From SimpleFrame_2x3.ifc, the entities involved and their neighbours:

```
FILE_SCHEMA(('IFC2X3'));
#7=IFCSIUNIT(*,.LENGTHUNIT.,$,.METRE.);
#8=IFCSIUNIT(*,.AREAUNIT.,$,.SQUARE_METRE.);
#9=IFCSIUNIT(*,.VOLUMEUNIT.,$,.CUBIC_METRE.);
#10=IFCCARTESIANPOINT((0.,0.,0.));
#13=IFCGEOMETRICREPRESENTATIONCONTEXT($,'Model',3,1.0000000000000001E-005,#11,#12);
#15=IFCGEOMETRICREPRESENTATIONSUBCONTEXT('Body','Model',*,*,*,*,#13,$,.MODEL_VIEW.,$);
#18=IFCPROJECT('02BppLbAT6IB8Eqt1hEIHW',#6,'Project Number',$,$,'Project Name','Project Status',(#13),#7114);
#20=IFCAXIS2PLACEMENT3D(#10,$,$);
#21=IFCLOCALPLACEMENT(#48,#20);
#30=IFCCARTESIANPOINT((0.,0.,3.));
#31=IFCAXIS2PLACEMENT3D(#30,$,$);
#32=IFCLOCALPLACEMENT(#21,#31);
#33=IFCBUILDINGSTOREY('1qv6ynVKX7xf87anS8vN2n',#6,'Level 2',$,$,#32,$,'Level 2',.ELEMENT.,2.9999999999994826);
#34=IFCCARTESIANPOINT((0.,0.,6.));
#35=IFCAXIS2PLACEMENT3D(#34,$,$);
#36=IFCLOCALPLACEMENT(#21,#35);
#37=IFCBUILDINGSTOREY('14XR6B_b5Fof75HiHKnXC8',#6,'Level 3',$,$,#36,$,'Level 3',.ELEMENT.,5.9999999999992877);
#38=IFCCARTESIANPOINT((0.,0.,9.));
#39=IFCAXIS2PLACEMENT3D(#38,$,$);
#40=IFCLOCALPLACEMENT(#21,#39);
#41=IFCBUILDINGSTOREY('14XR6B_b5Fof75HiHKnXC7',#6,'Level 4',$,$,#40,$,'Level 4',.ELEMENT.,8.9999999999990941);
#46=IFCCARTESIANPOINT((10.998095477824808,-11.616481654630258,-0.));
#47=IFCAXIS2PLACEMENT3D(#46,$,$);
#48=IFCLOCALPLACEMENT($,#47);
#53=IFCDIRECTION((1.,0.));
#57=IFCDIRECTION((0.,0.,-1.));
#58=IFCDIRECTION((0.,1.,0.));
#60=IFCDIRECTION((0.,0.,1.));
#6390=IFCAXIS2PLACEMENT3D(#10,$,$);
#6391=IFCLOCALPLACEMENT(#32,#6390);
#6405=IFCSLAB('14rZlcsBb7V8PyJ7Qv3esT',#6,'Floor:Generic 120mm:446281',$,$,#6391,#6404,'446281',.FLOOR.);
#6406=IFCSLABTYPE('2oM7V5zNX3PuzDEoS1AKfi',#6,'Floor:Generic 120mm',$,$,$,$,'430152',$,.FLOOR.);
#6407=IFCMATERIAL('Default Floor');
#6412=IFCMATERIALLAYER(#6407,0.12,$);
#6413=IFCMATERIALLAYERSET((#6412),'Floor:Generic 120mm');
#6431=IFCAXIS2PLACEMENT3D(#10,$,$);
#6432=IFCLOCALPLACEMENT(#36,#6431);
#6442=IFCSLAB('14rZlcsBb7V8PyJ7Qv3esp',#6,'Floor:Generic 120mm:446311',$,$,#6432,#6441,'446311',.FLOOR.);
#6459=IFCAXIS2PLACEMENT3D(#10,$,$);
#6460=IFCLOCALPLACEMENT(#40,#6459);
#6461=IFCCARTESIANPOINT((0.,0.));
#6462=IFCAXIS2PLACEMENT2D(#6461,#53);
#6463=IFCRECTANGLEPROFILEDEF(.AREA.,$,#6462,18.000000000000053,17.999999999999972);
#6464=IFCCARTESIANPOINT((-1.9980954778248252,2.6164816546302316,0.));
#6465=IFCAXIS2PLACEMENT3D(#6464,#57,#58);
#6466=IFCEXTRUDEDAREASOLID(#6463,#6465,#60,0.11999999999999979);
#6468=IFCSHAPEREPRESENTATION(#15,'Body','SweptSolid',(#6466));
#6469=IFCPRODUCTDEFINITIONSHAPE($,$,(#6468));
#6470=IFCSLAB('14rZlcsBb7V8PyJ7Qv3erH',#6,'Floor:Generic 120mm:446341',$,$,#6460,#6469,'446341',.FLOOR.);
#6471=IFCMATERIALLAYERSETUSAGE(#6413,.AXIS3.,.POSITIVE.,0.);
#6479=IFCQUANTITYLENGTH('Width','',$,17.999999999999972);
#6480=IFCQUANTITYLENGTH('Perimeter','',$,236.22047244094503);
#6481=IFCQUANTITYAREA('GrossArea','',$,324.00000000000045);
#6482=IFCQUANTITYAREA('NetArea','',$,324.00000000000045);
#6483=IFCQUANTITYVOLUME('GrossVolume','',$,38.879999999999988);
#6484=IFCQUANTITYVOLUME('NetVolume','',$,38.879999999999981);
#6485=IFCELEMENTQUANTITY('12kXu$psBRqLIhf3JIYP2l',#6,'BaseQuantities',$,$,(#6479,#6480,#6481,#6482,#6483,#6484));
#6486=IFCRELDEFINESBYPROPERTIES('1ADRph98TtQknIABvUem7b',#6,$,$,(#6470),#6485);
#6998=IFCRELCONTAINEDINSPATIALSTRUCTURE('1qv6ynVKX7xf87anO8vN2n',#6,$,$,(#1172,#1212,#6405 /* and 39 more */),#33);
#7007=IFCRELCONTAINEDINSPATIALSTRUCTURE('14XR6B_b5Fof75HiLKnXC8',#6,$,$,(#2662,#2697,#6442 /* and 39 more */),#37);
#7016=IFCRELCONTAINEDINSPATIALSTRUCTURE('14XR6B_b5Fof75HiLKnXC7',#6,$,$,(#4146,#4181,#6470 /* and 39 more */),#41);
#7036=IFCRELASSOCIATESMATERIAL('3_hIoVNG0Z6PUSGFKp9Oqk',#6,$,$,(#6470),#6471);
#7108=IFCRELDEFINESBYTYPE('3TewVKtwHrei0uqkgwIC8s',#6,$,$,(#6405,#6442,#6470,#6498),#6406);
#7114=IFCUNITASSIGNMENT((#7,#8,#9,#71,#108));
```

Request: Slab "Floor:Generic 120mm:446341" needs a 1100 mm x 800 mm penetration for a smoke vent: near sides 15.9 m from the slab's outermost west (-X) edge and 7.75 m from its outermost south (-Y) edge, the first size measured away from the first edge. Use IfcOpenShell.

```python
import numpy as np
import ifcopenshell
import ifcopenshell.api.feature
import ifcopenshell.api.geometry
import ifcopenshell.api.pset
import ifcopenshell.api.root
import ifcopenshell.geom
import ifcopenshell.util.element
import ifcopenshell.util.placement
import ifcopenshell.util.representation
import ifcopenshell.util.shape
import ifcopenshell.util.unit

model = ifcopenshell.open("SimpleFrame_2x3.ifc")
unit_scale = ifcopenshell.util.unit.calculate_unit_scale(model)
area_scale = ifcopenshell.util.unit.calculate_unit_scale(model, "AREAUNIT")
volume_scale = ifcopenshell.util.unit.calculate_unit_scale(model, "VOLUMEUNIT")
settings = ifcopenshell.geom.settings()


def volume(element):
    """Net volume in cubic metres, openings subtracted."""
    shape = ifcopenshell.geom.create_shape(settings, element)
    return ifcopenshell.util.shape.get_volume(shape.geometry)


slab = model.by_id(6470)
before = volume(slab)

# Extent in the slab's own axes, in metres. The edges named are its -X and -Y sides.
slab_shape = ifcopenshell.geom.create_shape(settings, slab)
vertices = ifcopenshell.util.shape.get_vertices(slab_shape.geometry)
x_min, y_min, bottom = vertices.min(axis=0)
top = vertices[:, 2].max()

opening = ifcopenshell.api.root.create_entity(model, ifc_class="IfcOpeningElement", name="Smoke vent opening")
context = ifcopenshell.util.representation.get_context(model, "Model", "Body", "MODEL_VIEW")
width, depth = 1.1, 0.8
outline = [(0.0, 0.0), (width, 0.0), (width, depth), (0.0, depth), (0.0, 0.0)]
# Overshoot both faces by 50 mm so the cut is clean.
shape = ifcopenshell.api.geometry.add_slab_representation(
    model, context=context, depth=top - bottom + 0.1, polyline=outline
)
ifcopenshell.api.geometry.assign_representation(model, product=opening, representation=shape)

matrix = ifcopenshell.util.placement.get_local_placement(slab.ObjectPlacement)
matrix[:, 3] = matrix @ np.append(np.array([x_min + 15.9, y_min + 7.75, bottom - 0.05]) / unit_scale, 1.0)
ifcopenshell.api.geometry.edit_object_placement(model, product=opening, matrix=matrix, is_si=False)
ifcopenshell.api.feature.add_feature(model, feature=opening, element=slab)

after = volume(slab)

# Update the slab's stored quantities.
qto = model.by_id(ifcopenshell.util.element.get_pset(slab, "BaseQuantities", should_inherit=False)["id"])
ifcopenshell.api.pset.edit_qto(model, qto=qto, properties={
    "NetArea": after / (top - bottom) / area_scale,
    "NetVolume": after / volume_scale,
})

print(f"slab volume {before:.3f} -> {after:.3f} m3")

model.write("SimpleFrame_2x3_edited.ifc")
```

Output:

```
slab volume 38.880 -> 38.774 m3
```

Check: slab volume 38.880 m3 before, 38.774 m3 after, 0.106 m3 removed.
